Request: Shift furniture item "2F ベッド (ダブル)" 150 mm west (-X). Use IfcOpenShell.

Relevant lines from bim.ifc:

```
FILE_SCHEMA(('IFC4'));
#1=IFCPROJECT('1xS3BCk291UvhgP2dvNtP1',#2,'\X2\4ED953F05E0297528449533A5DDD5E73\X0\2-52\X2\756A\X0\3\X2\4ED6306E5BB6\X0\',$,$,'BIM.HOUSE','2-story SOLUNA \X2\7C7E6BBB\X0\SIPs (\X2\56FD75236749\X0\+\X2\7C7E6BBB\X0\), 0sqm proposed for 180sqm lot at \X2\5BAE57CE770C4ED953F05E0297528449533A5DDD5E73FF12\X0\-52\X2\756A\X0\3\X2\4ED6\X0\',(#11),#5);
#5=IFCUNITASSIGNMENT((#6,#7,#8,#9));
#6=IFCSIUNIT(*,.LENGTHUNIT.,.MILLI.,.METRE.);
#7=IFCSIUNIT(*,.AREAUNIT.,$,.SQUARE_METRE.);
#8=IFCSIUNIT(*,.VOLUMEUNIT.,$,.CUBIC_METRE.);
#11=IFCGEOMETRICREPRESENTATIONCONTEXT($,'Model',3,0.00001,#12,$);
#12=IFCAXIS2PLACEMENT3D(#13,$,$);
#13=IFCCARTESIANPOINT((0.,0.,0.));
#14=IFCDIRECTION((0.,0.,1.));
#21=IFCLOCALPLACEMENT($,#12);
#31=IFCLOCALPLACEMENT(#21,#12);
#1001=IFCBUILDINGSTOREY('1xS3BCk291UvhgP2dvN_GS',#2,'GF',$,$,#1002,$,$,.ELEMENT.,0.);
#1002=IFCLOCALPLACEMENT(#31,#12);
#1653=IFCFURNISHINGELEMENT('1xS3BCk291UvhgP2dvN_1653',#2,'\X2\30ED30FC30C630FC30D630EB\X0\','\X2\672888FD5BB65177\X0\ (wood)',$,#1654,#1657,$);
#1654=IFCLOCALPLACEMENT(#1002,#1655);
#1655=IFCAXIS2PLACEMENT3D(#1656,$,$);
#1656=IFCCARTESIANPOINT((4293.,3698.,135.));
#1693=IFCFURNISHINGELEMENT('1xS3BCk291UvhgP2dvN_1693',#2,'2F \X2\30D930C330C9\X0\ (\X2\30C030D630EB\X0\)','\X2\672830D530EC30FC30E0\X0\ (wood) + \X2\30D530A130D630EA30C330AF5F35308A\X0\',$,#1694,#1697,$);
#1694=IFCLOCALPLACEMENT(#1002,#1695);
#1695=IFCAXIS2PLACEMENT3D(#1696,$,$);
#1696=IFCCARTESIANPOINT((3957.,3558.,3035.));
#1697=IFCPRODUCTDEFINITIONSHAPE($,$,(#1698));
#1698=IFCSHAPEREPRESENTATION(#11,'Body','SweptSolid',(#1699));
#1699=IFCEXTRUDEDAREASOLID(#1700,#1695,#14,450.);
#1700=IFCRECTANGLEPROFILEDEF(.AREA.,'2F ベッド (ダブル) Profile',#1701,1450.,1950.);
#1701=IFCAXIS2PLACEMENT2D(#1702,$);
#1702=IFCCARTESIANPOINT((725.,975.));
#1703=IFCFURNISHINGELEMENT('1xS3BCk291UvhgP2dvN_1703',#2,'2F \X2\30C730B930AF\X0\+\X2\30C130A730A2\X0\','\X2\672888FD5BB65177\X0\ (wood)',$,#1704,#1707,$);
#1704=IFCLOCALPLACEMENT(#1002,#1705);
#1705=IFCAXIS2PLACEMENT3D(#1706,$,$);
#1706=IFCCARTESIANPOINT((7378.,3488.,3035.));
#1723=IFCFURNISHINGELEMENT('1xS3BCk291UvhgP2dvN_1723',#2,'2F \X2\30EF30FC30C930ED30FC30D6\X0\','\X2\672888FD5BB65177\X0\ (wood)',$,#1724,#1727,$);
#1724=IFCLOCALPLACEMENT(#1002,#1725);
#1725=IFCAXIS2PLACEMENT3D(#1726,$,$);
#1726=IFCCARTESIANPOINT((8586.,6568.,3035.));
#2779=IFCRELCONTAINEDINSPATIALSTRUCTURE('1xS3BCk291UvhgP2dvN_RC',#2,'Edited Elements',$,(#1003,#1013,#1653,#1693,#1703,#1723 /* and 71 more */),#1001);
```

```python
import ifcopenshell
import ifcopenshell.api.geometry
import ifcopenshell.util.placement

model = ifcopenshell.open("bim.ifc")

item = model.by_guid("1xS3BCk291UvhgP2dvN_1693")
matrix = ifcopenshell.util.placement.get_local_placement(item.ObjectPlacement)
matrix[0, 3] -= 150.0
ifcopenshell.api.geometry.edit_object_placement(model, product=item, matrix=matrix, is_si=False)

print(ifcopenshell.util.placement.get_local_placement(item.ObjectPlacement).round(3) + 0.0)

model.write("bim-out.ifc")
```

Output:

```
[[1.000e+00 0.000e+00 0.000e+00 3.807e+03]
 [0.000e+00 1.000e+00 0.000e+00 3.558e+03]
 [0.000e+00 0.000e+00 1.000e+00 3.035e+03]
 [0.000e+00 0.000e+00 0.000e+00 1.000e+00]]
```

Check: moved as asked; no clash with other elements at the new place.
